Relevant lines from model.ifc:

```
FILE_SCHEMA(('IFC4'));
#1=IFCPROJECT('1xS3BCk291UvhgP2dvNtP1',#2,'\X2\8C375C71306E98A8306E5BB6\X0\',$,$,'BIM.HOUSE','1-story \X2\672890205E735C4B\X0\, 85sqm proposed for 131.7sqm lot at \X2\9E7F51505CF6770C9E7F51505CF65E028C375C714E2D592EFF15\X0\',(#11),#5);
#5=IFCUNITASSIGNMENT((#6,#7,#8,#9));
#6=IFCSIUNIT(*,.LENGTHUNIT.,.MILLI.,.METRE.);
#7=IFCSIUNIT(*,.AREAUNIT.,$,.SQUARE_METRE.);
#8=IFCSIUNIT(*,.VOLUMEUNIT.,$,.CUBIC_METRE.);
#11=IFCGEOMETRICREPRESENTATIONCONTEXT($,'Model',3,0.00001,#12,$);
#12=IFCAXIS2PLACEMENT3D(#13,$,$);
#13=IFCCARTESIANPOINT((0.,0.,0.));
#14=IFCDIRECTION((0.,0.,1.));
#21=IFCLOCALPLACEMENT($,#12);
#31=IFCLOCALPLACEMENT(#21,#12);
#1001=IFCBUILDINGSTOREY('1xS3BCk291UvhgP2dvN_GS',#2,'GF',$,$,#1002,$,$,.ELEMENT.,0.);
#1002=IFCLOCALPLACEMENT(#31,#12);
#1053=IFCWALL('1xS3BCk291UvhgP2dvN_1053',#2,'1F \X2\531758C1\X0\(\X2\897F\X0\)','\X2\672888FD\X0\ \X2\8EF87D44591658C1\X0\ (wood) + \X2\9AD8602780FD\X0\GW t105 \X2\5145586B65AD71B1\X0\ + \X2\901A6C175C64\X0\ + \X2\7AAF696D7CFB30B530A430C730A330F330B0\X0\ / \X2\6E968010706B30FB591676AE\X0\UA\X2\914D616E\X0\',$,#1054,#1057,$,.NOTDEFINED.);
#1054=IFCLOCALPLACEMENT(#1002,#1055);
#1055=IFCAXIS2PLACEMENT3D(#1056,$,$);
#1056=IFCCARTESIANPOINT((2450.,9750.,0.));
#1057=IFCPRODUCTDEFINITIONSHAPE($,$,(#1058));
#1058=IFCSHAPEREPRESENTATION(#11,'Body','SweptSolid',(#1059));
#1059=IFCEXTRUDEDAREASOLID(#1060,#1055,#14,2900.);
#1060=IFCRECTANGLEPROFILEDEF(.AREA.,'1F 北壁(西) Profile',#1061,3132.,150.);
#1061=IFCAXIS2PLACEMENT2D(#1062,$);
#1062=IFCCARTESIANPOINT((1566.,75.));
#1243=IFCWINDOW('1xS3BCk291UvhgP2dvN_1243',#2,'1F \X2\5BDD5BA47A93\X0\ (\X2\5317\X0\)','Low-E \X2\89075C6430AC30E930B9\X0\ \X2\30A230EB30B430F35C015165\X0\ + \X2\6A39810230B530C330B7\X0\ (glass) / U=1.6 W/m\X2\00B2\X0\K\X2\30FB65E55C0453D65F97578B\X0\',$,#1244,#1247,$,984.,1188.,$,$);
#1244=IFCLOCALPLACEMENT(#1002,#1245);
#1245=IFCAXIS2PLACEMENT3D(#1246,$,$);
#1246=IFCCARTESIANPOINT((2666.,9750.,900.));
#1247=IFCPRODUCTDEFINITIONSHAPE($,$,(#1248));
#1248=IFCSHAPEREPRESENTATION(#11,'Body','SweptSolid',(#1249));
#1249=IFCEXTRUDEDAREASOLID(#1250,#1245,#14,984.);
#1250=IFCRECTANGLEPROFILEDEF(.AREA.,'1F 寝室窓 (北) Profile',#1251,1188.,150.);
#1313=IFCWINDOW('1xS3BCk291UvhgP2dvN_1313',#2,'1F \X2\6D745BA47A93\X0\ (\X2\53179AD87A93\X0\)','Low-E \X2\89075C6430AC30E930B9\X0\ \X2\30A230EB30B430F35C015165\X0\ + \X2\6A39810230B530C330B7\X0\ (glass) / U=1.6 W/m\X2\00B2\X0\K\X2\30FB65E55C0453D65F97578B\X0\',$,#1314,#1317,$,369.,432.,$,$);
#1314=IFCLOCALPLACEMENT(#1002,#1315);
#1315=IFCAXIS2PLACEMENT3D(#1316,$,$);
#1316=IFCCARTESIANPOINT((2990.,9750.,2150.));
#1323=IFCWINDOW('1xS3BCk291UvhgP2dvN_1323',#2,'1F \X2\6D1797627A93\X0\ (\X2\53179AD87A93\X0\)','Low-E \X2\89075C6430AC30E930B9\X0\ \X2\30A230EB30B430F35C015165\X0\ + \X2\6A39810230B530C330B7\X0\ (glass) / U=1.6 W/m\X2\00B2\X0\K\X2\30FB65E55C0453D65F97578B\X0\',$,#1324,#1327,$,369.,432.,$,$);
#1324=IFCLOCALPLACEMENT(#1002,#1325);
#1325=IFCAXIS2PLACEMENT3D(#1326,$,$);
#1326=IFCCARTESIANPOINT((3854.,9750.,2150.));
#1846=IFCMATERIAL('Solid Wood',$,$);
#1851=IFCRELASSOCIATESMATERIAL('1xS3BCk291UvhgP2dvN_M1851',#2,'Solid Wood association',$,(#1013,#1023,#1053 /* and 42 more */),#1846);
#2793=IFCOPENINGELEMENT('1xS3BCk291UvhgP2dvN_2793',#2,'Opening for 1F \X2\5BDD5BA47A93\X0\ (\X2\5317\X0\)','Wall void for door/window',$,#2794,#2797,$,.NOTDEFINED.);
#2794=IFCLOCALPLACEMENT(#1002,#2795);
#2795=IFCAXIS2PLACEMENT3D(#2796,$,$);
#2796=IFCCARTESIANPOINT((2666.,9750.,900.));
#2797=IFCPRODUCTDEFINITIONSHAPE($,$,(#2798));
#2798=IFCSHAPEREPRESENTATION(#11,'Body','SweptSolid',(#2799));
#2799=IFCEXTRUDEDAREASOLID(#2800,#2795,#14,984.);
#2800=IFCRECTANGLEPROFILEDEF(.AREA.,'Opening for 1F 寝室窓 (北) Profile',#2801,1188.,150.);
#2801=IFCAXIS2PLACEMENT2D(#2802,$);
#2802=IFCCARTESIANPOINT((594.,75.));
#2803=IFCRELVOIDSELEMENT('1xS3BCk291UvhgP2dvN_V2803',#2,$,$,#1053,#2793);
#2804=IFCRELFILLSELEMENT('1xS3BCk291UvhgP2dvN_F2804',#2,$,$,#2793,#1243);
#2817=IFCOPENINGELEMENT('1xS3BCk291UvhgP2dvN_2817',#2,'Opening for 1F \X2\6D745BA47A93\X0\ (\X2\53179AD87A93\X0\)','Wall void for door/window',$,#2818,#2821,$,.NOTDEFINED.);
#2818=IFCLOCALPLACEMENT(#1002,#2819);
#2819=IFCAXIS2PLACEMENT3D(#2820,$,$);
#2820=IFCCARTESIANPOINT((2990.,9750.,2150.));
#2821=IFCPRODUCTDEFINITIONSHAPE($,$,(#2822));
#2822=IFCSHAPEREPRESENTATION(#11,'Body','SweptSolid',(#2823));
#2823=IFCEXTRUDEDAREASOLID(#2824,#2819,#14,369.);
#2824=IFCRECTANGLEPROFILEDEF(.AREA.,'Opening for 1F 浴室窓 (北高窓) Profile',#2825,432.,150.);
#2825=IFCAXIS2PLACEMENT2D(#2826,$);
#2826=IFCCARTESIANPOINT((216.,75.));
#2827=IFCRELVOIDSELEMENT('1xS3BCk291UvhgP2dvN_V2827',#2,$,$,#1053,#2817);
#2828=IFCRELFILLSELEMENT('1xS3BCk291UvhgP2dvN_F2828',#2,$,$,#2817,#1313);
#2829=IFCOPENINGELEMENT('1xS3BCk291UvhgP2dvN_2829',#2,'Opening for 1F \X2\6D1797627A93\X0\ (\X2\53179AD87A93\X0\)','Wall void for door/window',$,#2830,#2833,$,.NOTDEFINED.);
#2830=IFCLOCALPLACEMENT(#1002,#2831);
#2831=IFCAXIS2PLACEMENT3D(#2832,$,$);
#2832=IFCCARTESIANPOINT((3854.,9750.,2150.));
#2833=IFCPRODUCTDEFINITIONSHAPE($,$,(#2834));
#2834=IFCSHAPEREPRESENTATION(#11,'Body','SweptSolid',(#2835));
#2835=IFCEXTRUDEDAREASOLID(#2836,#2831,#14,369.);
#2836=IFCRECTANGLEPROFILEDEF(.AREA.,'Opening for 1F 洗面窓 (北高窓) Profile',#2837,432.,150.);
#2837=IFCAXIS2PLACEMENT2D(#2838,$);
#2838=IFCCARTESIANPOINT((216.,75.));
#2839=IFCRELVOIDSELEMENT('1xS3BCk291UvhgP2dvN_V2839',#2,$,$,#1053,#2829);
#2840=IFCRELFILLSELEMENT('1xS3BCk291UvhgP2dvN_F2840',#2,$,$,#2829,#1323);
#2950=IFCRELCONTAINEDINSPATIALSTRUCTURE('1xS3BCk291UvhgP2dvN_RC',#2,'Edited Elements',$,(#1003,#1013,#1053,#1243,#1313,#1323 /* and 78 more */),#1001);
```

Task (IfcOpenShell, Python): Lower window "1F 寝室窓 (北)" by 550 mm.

```python
import numpy as np
import ifcopenshell
import ifcopenshell.api.geometry
import ifcopenshell.util.placement
import ifcopenshell.util.unit

model = ifcopenshell.open("model.ifc")
unit_scale = ifcopenshell.util.unit.calculate_unit_scale(model)

window = model.by_guid("1xS3BCk291UvhgP2dvN_1243")
opening = window.FillsVoids[0].RelatingOpeningElement
dz = -0.55 / unit_scale

shift = np.array([0.0, 0.0, dz])
# The window is not placed relative to its opening, so move both.
for product in (opening, window):
    matrix = ifcopenshell.util.placement.get_local_placement(product.ObjectPlacement)
    matrix[:3, 3] += shift
    ifcopenshell.api.geometry.edit_object_placement(model, product=product, matrix=matrix, is_si=False)

print(f"moved by {dz * unit_scale:+.3f} m")

model.write("model_updated.ifc")
```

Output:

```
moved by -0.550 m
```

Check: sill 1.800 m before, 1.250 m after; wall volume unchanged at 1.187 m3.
